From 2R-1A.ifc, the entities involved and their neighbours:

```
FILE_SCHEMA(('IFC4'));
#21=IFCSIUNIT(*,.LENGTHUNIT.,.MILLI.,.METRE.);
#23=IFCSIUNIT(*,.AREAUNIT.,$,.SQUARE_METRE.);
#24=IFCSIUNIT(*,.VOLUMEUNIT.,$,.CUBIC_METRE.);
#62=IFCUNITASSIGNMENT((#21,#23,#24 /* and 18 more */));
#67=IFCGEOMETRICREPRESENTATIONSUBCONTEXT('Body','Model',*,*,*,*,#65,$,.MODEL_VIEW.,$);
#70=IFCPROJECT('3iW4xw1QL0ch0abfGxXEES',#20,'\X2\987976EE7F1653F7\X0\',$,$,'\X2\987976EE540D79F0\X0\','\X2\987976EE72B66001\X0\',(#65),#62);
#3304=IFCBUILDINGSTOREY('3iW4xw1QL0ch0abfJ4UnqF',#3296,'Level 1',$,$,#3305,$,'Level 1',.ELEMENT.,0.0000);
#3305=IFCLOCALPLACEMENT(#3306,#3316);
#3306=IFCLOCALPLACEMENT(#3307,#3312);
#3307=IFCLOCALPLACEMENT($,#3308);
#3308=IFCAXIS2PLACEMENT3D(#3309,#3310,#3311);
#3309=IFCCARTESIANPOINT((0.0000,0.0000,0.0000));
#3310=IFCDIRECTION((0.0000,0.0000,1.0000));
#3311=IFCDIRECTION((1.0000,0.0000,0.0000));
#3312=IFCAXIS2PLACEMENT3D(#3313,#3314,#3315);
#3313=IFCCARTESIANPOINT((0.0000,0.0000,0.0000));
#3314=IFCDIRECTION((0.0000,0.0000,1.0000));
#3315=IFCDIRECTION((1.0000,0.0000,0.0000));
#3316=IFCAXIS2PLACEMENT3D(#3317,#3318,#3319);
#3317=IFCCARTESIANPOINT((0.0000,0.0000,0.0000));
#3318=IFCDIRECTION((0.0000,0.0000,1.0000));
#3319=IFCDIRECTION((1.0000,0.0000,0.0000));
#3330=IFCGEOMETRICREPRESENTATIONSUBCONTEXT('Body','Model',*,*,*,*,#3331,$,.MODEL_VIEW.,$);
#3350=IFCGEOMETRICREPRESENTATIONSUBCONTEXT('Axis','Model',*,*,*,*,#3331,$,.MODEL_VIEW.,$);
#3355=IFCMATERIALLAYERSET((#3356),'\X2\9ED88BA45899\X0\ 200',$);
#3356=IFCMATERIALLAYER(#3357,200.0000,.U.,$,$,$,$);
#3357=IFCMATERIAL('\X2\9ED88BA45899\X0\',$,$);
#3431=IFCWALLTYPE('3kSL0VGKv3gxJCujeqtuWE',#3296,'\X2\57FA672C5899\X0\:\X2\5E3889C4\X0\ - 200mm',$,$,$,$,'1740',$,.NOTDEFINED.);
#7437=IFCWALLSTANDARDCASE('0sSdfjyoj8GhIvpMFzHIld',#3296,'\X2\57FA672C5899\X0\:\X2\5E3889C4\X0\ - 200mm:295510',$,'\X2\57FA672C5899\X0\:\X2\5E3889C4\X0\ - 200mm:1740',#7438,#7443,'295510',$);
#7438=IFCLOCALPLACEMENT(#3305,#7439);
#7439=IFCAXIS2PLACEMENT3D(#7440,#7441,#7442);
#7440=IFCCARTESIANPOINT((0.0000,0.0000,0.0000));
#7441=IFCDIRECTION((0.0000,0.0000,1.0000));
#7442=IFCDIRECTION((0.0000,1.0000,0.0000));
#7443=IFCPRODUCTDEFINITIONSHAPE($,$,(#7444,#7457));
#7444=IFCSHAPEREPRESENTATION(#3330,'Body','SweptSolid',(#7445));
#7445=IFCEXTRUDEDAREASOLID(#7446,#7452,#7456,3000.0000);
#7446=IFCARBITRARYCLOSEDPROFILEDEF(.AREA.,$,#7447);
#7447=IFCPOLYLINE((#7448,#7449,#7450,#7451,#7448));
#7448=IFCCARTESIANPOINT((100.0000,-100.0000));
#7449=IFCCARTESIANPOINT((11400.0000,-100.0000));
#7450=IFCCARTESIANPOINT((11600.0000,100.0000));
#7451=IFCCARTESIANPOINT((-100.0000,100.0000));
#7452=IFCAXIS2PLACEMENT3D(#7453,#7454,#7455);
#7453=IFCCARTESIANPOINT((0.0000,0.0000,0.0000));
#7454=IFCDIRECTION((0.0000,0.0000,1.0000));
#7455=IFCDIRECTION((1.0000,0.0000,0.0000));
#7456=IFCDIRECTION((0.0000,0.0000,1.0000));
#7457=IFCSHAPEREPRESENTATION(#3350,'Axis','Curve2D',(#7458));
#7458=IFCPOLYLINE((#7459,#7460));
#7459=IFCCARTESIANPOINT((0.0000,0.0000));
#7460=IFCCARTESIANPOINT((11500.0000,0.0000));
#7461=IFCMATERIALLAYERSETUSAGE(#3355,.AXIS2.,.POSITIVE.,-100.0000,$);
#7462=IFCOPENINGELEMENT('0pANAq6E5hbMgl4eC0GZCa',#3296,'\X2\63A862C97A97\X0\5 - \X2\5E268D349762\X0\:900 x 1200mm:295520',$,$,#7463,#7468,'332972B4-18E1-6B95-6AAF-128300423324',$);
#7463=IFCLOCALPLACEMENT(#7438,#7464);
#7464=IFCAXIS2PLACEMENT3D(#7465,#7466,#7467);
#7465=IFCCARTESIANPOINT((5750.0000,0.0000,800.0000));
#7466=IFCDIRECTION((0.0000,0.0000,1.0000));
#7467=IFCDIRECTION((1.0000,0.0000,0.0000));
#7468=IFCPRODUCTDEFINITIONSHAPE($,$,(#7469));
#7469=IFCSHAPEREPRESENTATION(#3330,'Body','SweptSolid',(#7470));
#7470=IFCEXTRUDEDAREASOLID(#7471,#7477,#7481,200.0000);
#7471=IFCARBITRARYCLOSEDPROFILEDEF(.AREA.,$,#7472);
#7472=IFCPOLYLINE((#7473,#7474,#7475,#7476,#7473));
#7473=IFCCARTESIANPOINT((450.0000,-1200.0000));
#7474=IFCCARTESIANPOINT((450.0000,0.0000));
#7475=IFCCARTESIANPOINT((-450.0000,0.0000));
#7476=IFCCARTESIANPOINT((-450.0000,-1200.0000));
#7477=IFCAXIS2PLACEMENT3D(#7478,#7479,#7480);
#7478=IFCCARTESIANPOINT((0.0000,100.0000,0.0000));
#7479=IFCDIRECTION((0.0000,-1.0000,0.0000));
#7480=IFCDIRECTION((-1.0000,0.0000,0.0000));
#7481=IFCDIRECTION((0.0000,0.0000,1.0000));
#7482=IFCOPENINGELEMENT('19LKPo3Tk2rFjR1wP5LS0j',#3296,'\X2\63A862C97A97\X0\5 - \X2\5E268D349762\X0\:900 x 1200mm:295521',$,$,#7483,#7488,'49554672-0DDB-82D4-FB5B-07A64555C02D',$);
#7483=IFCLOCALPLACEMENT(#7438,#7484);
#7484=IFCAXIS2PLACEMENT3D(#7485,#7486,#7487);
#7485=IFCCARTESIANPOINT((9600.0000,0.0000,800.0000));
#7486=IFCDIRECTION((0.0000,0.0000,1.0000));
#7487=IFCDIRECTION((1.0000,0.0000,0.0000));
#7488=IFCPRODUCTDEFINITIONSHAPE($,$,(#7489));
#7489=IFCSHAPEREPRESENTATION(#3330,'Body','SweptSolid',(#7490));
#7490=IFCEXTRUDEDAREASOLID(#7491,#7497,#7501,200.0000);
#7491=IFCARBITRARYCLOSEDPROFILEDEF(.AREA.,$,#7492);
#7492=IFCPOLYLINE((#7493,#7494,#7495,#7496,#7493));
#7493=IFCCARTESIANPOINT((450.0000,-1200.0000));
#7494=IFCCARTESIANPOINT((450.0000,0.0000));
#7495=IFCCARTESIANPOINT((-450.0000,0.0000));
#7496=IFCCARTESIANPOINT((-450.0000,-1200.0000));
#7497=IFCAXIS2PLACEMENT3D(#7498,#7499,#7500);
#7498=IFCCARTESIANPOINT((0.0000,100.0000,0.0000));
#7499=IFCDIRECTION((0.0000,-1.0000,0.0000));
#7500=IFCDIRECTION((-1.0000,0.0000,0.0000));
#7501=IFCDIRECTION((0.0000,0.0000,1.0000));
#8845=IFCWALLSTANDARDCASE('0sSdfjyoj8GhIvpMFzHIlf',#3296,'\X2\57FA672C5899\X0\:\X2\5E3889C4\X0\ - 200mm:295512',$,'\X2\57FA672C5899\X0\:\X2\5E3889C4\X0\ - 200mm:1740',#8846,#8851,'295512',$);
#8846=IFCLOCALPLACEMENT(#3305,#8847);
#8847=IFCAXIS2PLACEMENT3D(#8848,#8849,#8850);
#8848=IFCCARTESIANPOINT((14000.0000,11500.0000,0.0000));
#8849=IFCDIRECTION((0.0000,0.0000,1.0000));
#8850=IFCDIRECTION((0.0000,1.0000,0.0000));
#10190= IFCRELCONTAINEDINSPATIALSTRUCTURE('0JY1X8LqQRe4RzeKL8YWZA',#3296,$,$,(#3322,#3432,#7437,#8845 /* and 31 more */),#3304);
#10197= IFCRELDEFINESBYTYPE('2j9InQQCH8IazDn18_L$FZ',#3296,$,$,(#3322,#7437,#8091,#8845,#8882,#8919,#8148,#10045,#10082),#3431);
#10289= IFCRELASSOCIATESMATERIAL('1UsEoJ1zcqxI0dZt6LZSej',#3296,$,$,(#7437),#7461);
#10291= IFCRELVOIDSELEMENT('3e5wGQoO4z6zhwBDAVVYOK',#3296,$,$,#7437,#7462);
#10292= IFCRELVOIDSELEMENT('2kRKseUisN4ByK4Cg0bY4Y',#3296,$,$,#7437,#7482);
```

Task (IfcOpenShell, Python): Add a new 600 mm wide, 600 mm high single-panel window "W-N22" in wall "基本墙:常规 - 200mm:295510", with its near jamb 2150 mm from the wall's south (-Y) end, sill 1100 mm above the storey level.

```python
import numpy as np
import ifcopenshell
import ifcopenshell.api.feature
import ifcopenshell.api.geometry
import ifcopenshell.api.root
import ifcopenshell.api.spatial
import ifcopenshell.geom
import ifcopenshell.util.element
import ifcopenshell.util.placement
import ifcopenshell.util.representation
import ifcopenshell.util.shape
import ifcopenshell.util.unit

model = ifcopenshell.open("2R-1A.ifc")
unit_scale = ifcopenshell.util.unit.calculate_unit_scale(model)
settings = ifcopenshell.geom.settings()


def volume(element):
    """Net volume in cubic metres, openings subtracted."""
    shape = ifcopenshell.geom.create_shape(settings, element)
    return ifcopenshell.util.shape.get_volume(shape.geometry)


wall = model.by_guid("0sSdfjyoj8GhIvpMFzHIld")
storey = ifcopenshell.util.element.get_container(wall, ifc_class="IfcBuildingStorey")
context = ifcopenshell.util.representation.get_context(model, "Model", "Body", "MODEL_VIEW")
before = volume(wall)

width, height, from_end, sill = 0.6, 0.6, 2.15, 1.1  # metres

# The wall runs along its own X axis, and the end named is its -X end.
wall_shape = ifcopenshell.geom.create_shape(settings, wall)
x, y, z = ifcopenshell.util.shape.get_vertices(wall_shape.geometry).T
start = x.min() + from_end
face, thickness = float(y.min()), float(y.max() - y.min())
wall_matrix = ifcopenshell.util.placement.get_local_placement(wall.ObjectPlacement)
level = ifcopenshell.util.placement.get_local_placement(storey.ObjectPlacement)[2, 3]


def in_wall(x, y):
    """Placement at x, y metres in the wall's axes, at sill height."""
    matrix = wall_matrix.copy()
    matrix[:, 3] = wall_matrix @ np.array([x / unit_scale, y / unit_scale, 0.0, 1.0])
    matrix[2, 3] = level + sill / unit_scale
    return matrix


# Opening: a box that overshoots both wall faces by 50 mm.
opening = ifcopenshell.api.root.create_entity(model, ifc_class="IfcOpeningElement", predefined_type="OPENING")
box = ifcopenshell.api.geometry.add_wall_representation(
    model, context=context, length=width, height=height, thickness=thickness + 0.1
)
ifcopenshell.api.geometry.assign_representation(model, product=opening, representation=box)
ifcopenshell.api.geometry.edit_object_placement(model, product=opening, matrix=in_wall(start, face - 0.05), is_si=False)
ifcopenshell.api.feature.add_feature(model, feature=opening, element=wall)

window = ifcopenshell.api.root.create_entity(model, ifc_class="IfcWindow", name="W-N22", predefined_type="WINDOW")
window.OverallWidth, window.OverallHeight = width / unit_scale, height / unit_scale
window.PartitioningType = "SINGLE_PANEL"
body = ifcopenshell.api.geometry.add_window_representation(
    model,
    context=context,
    overall_width=window.OverallWidth,
    overall_height=window.OverallHeight,
    partition_type="SINGLE_PANEL",
)
ifcopenshell.api.geometry.assign_representation(model, product=window, representation=body)
ifcopenshell.api.spatial.assign_container(model, products=[window], relating_structure=storey)
ifcopenshell.api.feature.add_filling(model, opening=opening, element=window)

# Centre the window in the wall's thickness.
ifcopenshell.api.geometry.edit_object_placement(model, product=window, matrix=in_wall(start, face), is_si=False)
window_shape = ifcopenshell.geom.create_shape(settings, window)
depth = ifcopenshell.util.shape.get_vertices(window_shape.geometry)[:, 1]
offset = face + thickness / 2 - (depth.min() + depth.max()) / 2
ifcopenshell.api.geometry.edit_object_placement(model, product=window, matrix=in_wall(start, offset), is_si=False)

after = volume(wall)

print(f"wall volume {before:.3f} -> {after:.3f} m3")

model.write("2R-1A_updated.ifc")
```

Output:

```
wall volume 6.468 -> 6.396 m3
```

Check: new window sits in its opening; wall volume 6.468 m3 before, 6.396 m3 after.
